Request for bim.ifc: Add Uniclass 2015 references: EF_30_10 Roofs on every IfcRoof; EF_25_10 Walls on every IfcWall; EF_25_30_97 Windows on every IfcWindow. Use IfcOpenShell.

First a look at what the model holds.

```python
import ifcopenshell

model = ifcopenshell.open("bim.ifc")
print(model.schema)
print("classifications:", [c.Name for c in model.by_type("IfcClassification")])
for ifc_class in ("IfcDoor", "IfcRoof", "IfcStair", "IfcWall", "IfcWindow"):
    print(ifc_class, len(model.by_type(ifc_class)))
```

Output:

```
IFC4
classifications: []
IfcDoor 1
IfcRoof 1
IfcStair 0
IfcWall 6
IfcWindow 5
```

```python
import ifcopenshell
import ifcopenshell.api.classification

model = ifcopenshell.open("bim.ifc")

system = ifcopenshell.api.classification.add_classification(model, classification="Uniclass 2015")

codes = {
    "IfcRoof": ("EF_30_10", "Roofs"),
    "IfcWall": ("EF_25_10", "Walls"),
    "IfcWindow": ("EF_25_30_97", "Windows"),
}
for ifc_class, (code, name) in codes.items():
    products = model.by_type(ifc_class)
    ifcopenshell.api.classification.add_reference(
        model, products=products, classification=system, identification=code, name=name
    )
    print(code, len(products))

model.write("bim_rev.ifc")
```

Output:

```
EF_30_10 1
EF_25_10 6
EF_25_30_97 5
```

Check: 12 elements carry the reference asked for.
